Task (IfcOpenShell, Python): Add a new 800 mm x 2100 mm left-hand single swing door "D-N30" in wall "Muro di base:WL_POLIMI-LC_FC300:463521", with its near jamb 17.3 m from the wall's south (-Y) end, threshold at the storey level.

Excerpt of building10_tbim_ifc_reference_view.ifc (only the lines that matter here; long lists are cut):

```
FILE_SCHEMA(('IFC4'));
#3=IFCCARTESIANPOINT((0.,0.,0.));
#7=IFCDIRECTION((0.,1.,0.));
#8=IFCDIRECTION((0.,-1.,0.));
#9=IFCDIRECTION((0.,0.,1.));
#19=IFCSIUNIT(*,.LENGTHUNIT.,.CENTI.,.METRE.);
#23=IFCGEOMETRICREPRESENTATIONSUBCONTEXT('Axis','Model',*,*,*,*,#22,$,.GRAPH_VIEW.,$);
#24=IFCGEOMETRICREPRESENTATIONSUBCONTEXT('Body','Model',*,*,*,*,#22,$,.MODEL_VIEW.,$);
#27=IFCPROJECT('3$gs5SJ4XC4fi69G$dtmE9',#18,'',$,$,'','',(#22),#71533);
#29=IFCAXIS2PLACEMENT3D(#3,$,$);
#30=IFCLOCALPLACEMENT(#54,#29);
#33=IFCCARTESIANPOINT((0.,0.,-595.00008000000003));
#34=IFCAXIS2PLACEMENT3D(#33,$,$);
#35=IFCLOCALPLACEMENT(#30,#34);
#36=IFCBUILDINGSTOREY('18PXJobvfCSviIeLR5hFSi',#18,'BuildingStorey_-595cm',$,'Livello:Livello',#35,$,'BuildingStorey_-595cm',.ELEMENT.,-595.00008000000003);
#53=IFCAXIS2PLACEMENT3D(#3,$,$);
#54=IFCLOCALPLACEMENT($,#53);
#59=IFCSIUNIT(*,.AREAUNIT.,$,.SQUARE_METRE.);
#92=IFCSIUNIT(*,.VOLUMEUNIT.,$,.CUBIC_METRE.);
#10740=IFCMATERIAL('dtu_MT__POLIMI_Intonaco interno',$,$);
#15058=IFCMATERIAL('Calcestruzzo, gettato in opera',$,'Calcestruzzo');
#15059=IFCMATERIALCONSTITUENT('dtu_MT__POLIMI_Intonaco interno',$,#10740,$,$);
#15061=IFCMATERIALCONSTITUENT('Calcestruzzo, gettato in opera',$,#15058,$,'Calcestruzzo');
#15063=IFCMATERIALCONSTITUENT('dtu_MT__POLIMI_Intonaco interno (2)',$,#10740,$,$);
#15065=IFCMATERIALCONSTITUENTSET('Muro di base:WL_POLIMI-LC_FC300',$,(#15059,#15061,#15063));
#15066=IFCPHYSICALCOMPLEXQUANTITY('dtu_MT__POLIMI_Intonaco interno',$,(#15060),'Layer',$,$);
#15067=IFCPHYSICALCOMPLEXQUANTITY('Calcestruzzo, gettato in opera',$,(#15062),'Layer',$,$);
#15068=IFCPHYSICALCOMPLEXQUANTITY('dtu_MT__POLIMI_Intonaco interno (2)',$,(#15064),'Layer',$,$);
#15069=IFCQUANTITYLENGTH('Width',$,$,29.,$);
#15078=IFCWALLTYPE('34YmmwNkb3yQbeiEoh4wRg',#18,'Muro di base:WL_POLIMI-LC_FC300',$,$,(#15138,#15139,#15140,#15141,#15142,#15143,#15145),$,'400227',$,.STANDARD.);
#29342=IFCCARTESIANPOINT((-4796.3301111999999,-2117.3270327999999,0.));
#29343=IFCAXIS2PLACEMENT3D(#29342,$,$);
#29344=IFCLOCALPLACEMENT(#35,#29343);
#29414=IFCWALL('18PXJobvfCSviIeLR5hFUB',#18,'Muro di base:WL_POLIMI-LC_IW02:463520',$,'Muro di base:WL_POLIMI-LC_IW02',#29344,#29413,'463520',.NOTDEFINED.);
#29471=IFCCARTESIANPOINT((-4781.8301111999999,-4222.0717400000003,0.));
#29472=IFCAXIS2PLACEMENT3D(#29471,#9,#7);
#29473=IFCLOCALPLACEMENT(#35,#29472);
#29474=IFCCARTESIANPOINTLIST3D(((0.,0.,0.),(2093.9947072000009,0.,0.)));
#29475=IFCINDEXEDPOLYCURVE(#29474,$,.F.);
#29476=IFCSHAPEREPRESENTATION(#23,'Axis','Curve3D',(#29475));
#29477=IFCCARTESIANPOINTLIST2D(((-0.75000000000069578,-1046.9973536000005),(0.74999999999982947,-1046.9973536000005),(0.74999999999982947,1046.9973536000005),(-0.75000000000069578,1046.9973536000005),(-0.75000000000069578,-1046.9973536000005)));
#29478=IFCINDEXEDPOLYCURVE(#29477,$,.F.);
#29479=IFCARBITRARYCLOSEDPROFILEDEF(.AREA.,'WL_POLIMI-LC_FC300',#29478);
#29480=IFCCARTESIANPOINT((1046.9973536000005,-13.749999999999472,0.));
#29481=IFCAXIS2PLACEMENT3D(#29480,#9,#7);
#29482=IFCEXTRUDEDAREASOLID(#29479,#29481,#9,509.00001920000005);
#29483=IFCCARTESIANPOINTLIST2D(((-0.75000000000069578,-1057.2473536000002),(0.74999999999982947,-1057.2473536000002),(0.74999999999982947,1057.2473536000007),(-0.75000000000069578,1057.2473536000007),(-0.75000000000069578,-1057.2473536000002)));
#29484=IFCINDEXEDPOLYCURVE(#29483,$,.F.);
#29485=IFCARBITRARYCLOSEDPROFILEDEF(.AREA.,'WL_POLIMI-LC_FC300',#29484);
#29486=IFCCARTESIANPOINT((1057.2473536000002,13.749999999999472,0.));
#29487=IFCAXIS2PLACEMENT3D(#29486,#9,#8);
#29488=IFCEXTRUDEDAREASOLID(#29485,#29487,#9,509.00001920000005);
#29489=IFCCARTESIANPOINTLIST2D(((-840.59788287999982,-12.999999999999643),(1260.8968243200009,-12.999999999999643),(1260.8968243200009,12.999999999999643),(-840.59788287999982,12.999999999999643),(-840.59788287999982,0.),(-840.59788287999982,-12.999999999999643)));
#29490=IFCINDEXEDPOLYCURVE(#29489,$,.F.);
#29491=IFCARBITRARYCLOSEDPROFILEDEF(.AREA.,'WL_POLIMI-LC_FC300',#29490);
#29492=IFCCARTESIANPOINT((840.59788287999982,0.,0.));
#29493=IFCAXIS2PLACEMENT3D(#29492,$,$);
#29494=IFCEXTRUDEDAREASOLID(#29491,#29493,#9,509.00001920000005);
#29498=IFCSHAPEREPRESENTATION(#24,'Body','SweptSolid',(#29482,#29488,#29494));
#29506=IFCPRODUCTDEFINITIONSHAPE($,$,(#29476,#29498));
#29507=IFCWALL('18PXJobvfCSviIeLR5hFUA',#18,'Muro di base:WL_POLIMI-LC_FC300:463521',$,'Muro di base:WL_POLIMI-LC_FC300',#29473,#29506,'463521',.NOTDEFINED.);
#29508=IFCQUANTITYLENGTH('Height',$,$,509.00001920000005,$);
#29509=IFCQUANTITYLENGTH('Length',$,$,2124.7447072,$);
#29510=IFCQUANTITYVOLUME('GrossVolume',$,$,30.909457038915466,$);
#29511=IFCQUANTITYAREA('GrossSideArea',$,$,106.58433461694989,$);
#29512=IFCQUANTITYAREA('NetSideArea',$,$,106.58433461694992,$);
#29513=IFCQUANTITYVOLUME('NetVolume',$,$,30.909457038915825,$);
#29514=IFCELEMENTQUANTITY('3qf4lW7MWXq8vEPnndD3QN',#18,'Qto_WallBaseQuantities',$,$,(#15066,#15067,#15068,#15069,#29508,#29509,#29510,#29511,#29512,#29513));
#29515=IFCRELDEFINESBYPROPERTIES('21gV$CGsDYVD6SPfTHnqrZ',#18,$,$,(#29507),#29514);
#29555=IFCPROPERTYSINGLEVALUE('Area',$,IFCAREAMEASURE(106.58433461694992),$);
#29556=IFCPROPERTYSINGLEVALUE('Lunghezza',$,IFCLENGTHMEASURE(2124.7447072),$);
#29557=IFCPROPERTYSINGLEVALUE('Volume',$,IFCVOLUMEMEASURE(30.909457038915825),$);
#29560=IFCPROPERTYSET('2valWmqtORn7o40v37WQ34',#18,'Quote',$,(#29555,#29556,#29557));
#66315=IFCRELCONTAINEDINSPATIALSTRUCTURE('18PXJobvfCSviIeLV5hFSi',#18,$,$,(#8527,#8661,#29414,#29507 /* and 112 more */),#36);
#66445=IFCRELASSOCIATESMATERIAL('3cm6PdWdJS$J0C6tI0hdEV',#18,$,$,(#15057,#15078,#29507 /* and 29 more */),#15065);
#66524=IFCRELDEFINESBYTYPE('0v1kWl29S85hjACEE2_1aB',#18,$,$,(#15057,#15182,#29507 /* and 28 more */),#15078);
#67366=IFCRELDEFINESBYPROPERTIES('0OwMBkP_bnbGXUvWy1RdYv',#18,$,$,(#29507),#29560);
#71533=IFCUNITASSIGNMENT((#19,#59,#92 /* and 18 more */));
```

```python
import numpy as np
import ifcopenshell
import ifcopenshell.api.feature
import ifcopenshell.api.geometry
import ifcopenshell.api.pset
import ifcopenshell.api.root
import ifcopenshell.api.spatial
import ifcopenshell.geom
import ifcopenshell.util.element
import ifcopenshell.util.placement
import ifcopenshell.util.representation
import ifcopenshell.util.shape
import ifcopenshell.util.unit

model = ifcopenshell.open("building10_tbim_ifc_reference_view.ifc")
unit_scale = ifcopenshell.util.unit.calculate_unit_scale(model)
area_scale = ifcopenshell.util.unit.calculate_unit_scale(model, "AREAUNIT")
volume_scale = ifcopenshell.util.unit.calculate_unit_scale(model, "VOLUMEUNIT")
settings = ifcopenshell.geom.settings()


def volume(element):
    """Net volume in cubic metres, openings subtracted."""
    shape = ifcopenshell.geom.create_shape(settings, element)
    return ifcopenshell.util.shape.get_volume(shape.geometry)


wall = model.by_id(29507)
storey = ifcopenshell.util.element.get_container(wall, ifc_class="IfcBuildingStorey")
context = ifcopenshell.util.representation.get_context(model, "Model", "Body", "MODEL_VIEW")
before = volume(wall)

width, height, from_end, sill = 0.8, 2.1, 17.3, 0.0  # metres

# The wall runs along its own X axis, and the end named is its -X end.
wall_shape = ifcopenshell.geom.create_shape(settings, wall)
x, y, z = ifcopenshell.util.shape.get_vertices(wall_shape.geometry).T
start = x.min() + from_end
face, thickness = float(y.min()), float(y.max() - y.min())
wall_matrix = ifcopenshell.util.placement.get_local_placement(wall.ObjectPlacement)
level = ifcopenshell.util.placement.get_local_placement(storey.ObjectPlacement)[2, 3]


def in_wall(x, y):
    """Placement at x, y metres in the wall's axes, at sill height."""
    matrix = wall_matrix.copy()
    matrix[:, 3] = wall_matrix @ np.array([x / unit_scale, y / unit_scale, 0.0, 1.0])
    matrix[2, 3] = level + sill / unit_scale
    return matrix


# Opening: a box that overshoots both wall faces by 50 mm.
opening = ifcopenshell.api.root.create_entity(model, ifc_class="IfcOpeningElement", predefined_type="OPENING")
box = ifcopenshell.api.geometry.add_wall_representation(
    model, context=context, length=width, height=height, thickness=thickness + 0.1
)
ifcopenshell.api.geometry.assign_representation(model, product=opening, representation=box)
ifcopenshell.api.geometry.edit_object_placement(model, product=opening, matrix=in_wall(start, face - 0.05), is_si=False)
ifcopenshell.api.feature.add_feature(model, feature=opening, element=wall)

door = ifcopenshell.api.root.create_entity(model, ifc_class="IfcDoor", name="D-N30", predefined_type="DOOR")
door.OverallWidth, door.OverallHeight = width / unit_scale, height / unit_scale
door.OperationType = "SINGLE_SWING_LEFT"
body = ifcopenshell.api.geometry.add_door_representation(
    model,
    context=context,
    overall_width=door.OverallWidth,
    overall_height=door.OverallHeight,
    operation_type="SINGLE_SWING_LEFT",
    lining_properties={"LiningDepth": thickness / unit_scale, "ThresholdDepth": thickness / unit_scale},
)
ifcopenshell.api.geometry.assign_representation(model, product=door, representation=body)
ifcopenshell.api.spatial.assign_container(model, products=[door], relating_structure=storey)
ifcopenshell.api.feature.add_filling(model, opening=opening, element=door)

# The lining spans the wall, so the door starts at the wall face.
ifcopenshell.api.geometry.edit_object_placement(model, product=door, matrix=in_wall(start, face), is_si=False)

after = volume(wall)

# Update the wall's stored quantities.
qto = model.by_id(ifcopenshell.util.element.get_pset(wall, "Qto_WallBaseQuantities", should_inherit=False)["id"])
ifcopenshell.api.pset.edit_qto(model, qto=qto, properties={
    "NetSideArea": after / thickness / area_scale,
    "NetVolume": after / volume_scale,
})
pset = model.by_id(ifcopenshell.util.element.get_pset(wall, "Quote", should_inherit=False)["id"])
ifcopenshell.api.pset.edit_pset(model, pset=pset, properties={
    "Area": model.create_entity("IfcAreaMeasure", after / thickness / area_scale),
    "Volume": model.create_entity("IfcVolumeMeasure", after / volume_scale),
})

print(f"wall volume {before:.3f} -> {after:.3f} m3")

model.write("building10_tbim_ifc_reference_view-out.ifc")
```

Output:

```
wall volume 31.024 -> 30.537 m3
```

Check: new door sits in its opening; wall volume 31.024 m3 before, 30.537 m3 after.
